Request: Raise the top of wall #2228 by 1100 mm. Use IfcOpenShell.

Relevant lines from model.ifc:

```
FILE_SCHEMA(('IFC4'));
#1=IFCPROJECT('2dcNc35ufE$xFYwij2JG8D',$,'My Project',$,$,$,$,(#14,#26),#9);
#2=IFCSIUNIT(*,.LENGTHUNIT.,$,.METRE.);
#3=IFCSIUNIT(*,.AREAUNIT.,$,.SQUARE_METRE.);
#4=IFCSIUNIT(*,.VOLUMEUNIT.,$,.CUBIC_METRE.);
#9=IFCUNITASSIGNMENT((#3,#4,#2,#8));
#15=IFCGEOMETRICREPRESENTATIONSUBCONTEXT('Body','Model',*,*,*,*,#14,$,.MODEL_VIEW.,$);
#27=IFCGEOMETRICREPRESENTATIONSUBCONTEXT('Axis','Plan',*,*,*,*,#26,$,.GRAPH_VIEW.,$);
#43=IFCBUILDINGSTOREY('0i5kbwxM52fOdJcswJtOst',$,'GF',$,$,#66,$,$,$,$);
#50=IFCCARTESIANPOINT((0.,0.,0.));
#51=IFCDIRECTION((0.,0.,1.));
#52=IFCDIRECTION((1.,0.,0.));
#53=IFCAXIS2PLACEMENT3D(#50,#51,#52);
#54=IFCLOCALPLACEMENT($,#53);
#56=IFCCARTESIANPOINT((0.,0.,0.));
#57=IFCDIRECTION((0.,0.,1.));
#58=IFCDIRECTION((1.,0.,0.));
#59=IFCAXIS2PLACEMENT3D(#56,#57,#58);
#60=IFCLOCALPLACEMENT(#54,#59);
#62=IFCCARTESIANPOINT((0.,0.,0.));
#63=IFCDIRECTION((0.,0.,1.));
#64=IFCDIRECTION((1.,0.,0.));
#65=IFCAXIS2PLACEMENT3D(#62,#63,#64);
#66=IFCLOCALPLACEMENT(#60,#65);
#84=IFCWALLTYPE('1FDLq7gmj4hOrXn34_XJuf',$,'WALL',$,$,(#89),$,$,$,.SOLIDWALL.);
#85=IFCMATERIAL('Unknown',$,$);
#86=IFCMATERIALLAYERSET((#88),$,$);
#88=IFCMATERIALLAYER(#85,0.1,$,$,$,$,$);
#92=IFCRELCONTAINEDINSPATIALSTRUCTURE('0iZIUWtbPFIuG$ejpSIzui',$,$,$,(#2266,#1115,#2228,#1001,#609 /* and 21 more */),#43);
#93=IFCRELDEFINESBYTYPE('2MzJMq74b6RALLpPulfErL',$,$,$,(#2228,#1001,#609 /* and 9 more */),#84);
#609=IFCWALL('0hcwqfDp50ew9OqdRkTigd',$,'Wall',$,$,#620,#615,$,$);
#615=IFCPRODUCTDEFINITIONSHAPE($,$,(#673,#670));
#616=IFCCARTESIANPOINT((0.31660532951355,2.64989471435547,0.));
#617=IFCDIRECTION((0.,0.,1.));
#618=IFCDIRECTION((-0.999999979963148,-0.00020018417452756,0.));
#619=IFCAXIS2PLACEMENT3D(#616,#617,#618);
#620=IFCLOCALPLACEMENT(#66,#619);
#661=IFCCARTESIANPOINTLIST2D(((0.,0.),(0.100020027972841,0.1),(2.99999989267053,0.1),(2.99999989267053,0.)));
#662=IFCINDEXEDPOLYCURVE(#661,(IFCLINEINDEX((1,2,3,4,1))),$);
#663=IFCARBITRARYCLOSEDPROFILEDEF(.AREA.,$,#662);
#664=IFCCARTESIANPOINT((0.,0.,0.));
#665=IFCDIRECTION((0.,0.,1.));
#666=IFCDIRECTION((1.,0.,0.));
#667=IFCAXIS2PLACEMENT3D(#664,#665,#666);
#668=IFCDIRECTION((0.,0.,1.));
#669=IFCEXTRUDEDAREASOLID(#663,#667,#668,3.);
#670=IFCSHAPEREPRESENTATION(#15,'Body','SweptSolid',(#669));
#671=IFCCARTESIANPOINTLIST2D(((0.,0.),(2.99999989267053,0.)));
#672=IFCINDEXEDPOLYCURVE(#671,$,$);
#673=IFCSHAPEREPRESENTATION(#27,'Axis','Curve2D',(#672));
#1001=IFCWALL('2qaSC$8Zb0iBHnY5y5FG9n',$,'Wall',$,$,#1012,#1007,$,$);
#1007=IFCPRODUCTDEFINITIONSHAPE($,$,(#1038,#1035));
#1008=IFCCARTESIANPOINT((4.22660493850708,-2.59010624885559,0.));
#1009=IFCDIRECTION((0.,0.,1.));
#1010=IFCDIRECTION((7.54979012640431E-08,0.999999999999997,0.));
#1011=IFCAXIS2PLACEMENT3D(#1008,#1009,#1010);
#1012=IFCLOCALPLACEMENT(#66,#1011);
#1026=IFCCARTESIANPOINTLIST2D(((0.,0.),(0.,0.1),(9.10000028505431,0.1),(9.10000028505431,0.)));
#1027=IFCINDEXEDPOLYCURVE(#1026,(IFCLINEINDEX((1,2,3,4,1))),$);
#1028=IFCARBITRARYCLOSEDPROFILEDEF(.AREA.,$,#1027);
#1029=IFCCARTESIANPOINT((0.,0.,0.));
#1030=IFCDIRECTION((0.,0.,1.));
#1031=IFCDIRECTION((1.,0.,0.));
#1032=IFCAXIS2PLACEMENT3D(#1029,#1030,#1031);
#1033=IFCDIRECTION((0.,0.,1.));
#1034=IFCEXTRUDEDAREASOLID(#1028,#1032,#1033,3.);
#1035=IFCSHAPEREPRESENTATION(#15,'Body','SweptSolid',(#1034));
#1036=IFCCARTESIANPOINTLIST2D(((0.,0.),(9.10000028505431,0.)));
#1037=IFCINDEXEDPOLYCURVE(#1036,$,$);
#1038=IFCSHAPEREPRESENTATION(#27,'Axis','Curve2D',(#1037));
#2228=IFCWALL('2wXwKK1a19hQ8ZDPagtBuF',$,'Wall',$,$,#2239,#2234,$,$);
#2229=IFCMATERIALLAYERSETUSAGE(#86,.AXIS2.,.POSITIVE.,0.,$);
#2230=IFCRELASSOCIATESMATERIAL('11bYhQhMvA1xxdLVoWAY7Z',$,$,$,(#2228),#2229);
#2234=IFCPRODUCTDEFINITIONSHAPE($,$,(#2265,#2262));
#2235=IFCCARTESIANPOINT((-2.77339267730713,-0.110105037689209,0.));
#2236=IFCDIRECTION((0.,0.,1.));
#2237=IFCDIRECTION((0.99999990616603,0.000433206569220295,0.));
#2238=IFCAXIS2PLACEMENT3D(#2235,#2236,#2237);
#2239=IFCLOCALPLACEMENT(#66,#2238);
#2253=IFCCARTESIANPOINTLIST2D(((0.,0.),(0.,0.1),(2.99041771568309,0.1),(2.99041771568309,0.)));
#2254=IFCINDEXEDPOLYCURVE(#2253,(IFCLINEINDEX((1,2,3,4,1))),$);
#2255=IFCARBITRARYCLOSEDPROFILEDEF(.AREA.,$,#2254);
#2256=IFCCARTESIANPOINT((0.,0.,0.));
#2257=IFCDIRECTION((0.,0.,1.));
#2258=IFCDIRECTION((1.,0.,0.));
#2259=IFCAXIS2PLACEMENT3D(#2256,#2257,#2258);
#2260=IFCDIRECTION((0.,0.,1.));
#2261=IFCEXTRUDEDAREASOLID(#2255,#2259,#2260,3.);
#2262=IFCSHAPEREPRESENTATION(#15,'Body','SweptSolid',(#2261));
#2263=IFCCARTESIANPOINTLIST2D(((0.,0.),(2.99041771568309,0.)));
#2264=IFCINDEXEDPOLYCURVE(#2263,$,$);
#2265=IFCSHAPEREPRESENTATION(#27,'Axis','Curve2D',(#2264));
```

```python
import ifcopenshell
import ifcopenshell.geom
import ifcopenshell.util.representation
import ifcopenshell.util.shape

model = ifcopenshell.open("model.ifc")
settings = ifcopenshell.geom.settings()


def volume(element):
    """Net volume in cubic metres, openings subtracted."""
    shape = ifcopenshell.geom.create_shape(settings, element)
    return ifcopenshell.util.shape.get_volume(shape.geometry)


wall = model.by_id(2228)
before = volume(wall)

body = ifcopenshell.util.representation.get_representation(wall, "Model", "Body")
solid = body.Items[0]
old_height = solid.Depth
solid.Depth += 1.1
after = volume(wall)

print(f"height {old_height:g} -> {solid.Depth:g}, volume {before:.3f} -> {after:.3f} m3")

model.write("model_v2.ifc")
```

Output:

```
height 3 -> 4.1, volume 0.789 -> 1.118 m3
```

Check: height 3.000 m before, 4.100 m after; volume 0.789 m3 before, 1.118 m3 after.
